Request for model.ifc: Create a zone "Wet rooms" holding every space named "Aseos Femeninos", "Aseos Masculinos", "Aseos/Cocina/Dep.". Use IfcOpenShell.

First a look at what the model holds.

```python
import ifcopenshell

model = ifcopenshell.open("model.ifc")
print(model.schema)
seen = {}
for space in model.by_type("IfcSpace"):
    seen[space.LongName] = seen.get(space.LongName, 0) + 1
for name, count in sorted(seen.items(), key=str):
    print(count, "x", name)
print("zones:", [z.Name for z in model.by_type("IfcZone")][:20])
```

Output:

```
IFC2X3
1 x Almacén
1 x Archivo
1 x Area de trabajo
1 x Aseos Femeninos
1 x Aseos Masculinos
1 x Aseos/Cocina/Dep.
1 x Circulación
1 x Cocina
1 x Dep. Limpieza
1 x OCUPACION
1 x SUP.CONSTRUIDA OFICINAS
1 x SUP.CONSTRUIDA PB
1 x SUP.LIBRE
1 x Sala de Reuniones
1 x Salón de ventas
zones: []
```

```python
import ifcopenshell
import ifcopenshell.api.group
import ifcopenshell.api.root

model = ifcopenshell.open("model.ifc")

names = {"Aseos Femeninos", "Aseos Masculinos", "Aseos/Cocina/Dep."}
spaces = [s for s in model.by_type("IfcSpace") if s.LongName in names]

zone = ifcopenshell.api.root.create_entity(model, ifc_class="IfcZone", name="Wet rooms")
ifcopenshell.api.group.assign_group(model, products=spaces, group=zone)
print(len(spaces), "spaces in", zone.Name)

model.write("model-out.ifc")
```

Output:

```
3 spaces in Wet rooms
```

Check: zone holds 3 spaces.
